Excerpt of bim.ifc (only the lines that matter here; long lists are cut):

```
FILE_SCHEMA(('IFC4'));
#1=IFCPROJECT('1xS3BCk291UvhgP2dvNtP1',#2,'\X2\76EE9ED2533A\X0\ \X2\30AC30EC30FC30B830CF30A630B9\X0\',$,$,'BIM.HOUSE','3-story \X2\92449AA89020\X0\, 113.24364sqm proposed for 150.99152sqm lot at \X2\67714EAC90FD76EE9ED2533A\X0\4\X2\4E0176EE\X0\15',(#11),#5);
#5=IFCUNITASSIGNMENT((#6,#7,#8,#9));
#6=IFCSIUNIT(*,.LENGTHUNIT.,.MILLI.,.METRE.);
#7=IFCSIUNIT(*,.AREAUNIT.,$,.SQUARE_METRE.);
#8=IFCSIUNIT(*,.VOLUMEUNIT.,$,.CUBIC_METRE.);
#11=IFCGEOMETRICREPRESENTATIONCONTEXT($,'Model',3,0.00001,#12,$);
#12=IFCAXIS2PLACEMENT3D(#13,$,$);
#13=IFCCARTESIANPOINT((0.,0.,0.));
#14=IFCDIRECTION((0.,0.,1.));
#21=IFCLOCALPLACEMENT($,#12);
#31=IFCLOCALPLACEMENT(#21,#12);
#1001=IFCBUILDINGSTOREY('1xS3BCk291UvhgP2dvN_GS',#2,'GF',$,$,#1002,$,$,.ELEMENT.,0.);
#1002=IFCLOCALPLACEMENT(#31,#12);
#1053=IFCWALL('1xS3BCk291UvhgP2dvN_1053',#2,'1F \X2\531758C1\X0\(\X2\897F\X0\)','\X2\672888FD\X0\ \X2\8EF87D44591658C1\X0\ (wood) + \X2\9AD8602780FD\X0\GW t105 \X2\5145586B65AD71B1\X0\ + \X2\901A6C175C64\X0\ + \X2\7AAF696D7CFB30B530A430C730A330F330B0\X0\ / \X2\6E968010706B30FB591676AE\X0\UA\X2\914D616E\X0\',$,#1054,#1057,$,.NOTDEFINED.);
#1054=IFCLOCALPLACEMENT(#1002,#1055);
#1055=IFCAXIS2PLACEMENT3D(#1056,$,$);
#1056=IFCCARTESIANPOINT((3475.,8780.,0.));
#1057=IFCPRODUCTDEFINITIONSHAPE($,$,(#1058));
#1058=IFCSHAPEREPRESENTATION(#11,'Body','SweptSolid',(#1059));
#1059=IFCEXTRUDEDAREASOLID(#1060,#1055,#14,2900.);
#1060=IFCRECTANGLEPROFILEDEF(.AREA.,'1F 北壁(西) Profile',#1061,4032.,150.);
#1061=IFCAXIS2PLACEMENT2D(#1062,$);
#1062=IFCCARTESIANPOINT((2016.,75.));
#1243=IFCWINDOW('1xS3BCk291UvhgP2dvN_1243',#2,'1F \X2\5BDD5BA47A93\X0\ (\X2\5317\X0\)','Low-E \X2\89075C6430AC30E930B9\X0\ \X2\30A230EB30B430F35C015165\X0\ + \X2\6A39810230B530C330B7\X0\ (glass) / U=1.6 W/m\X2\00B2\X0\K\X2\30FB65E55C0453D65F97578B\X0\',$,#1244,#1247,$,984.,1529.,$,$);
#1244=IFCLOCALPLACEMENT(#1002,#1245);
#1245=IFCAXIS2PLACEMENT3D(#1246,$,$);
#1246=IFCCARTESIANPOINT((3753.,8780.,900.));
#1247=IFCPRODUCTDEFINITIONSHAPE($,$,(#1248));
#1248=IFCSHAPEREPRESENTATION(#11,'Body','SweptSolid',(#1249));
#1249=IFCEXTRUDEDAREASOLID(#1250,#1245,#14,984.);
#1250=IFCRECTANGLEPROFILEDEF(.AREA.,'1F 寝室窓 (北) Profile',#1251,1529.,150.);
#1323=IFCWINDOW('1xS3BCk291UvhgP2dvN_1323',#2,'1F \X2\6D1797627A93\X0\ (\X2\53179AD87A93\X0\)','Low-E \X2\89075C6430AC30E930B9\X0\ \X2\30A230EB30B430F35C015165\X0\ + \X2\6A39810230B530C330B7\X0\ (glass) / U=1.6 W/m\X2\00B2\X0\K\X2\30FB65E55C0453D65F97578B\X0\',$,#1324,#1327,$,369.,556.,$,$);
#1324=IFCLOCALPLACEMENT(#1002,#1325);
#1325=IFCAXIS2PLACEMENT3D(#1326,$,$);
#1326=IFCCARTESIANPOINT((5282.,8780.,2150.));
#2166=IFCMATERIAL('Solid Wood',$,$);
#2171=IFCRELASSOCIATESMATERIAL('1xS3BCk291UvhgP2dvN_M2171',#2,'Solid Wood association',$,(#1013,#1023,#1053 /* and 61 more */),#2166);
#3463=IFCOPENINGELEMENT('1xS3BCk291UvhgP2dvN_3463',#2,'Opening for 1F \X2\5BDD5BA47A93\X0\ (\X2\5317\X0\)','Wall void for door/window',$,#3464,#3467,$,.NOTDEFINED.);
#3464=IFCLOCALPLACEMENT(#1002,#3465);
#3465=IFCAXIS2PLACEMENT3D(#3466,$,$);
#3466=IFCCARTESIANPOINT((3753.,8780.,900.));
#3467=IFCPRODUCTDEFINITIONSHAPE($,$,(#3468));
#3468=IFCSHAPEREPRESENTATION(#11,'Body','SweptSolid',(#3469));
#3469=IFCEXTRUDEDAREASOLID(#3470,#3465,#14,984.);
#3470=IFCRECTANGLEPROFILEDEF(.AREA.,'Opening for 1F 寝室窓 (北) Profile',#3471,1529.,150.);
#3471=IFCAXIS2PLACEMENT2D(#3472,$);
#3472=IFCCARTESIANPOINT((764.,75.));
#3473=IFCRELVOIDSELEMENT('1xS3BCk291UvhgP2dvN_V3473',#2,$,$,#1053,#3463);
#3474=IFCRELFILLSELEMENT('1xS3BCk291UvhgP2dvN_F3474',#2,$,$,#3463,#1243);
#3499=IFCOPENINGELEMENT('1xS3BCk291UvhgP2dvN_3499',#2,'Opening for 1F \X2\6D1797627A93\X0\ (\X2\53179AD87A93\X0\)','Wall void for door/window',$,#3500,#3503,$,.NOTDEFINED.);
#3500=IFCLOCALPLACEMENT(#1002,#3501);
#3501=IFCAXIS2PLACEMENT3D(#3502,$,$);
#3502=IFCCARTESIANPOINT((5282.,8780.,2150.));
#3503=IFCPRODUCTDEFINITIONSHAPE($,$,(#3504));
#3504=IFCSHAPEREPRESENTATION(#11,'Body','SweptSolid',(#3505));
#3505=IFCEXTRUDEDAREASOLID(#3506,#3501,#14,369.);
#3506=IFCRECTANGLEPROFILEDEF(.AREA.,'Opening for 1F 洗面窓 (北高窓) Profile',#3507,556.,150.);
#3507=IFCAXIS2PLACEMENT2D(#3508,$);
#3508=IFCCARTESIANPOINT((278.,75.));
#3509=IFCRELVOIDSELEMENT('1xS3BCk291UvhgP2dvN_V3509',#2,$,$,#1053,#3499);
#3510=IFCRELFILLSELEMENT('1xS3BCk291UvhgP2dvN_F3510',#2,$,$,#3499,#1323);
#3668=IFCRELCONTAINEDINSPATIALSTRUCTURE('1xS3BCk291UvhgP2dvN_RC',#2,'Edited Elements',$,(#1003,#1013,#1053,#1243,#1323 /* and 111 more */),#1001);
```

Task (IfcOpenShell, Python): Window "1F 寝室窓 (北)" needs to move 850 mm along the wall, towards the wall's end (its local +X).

```python
import ifcopenshell
import ifcopenshell.api.geometry
import ifcopenshell.util.placement

model = ifcopenshell.open("bim.ifc")

window = model.by_guid("1xS3BCk291UvhgP2dvN_1243")
opening = window.FillsVoids[0].RelatingOpeningElement
wall = opening.VoidsElements[0].RelatingBuildingElement

wall_matrix = ifcopenshell.util.placement.get_local_placement(wall.ObjectPlacement)
shift = wall_matrix[:3, 0] * 850.0
before = ifcopenshell.util.placement.get_local_placement(window.ObjectPlacement)[:3, 3].copy()

# The window is not placed relative to its opening, so move both.
for product in (opening, window):
    matrix = ifcopenshell.util.placement.get_local_placement(product.ObjectPlacement)
    matrix[:3, 3] += shift
    ifcopenshell.api.geometry.edit_object_placement(model, product=product, matrix=matrix, is_si=False)

after = ifcopenshell.util.placement.get_local_placement(window.ObjectPlacement)[:3, 3]
print("window moved by", (after - before).round(3) + 0.0)

model.write("bim-out.ifc")
```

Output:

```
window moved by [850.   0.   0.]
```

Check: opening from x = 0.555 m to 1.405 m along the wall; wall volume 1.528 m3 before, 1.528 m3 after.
